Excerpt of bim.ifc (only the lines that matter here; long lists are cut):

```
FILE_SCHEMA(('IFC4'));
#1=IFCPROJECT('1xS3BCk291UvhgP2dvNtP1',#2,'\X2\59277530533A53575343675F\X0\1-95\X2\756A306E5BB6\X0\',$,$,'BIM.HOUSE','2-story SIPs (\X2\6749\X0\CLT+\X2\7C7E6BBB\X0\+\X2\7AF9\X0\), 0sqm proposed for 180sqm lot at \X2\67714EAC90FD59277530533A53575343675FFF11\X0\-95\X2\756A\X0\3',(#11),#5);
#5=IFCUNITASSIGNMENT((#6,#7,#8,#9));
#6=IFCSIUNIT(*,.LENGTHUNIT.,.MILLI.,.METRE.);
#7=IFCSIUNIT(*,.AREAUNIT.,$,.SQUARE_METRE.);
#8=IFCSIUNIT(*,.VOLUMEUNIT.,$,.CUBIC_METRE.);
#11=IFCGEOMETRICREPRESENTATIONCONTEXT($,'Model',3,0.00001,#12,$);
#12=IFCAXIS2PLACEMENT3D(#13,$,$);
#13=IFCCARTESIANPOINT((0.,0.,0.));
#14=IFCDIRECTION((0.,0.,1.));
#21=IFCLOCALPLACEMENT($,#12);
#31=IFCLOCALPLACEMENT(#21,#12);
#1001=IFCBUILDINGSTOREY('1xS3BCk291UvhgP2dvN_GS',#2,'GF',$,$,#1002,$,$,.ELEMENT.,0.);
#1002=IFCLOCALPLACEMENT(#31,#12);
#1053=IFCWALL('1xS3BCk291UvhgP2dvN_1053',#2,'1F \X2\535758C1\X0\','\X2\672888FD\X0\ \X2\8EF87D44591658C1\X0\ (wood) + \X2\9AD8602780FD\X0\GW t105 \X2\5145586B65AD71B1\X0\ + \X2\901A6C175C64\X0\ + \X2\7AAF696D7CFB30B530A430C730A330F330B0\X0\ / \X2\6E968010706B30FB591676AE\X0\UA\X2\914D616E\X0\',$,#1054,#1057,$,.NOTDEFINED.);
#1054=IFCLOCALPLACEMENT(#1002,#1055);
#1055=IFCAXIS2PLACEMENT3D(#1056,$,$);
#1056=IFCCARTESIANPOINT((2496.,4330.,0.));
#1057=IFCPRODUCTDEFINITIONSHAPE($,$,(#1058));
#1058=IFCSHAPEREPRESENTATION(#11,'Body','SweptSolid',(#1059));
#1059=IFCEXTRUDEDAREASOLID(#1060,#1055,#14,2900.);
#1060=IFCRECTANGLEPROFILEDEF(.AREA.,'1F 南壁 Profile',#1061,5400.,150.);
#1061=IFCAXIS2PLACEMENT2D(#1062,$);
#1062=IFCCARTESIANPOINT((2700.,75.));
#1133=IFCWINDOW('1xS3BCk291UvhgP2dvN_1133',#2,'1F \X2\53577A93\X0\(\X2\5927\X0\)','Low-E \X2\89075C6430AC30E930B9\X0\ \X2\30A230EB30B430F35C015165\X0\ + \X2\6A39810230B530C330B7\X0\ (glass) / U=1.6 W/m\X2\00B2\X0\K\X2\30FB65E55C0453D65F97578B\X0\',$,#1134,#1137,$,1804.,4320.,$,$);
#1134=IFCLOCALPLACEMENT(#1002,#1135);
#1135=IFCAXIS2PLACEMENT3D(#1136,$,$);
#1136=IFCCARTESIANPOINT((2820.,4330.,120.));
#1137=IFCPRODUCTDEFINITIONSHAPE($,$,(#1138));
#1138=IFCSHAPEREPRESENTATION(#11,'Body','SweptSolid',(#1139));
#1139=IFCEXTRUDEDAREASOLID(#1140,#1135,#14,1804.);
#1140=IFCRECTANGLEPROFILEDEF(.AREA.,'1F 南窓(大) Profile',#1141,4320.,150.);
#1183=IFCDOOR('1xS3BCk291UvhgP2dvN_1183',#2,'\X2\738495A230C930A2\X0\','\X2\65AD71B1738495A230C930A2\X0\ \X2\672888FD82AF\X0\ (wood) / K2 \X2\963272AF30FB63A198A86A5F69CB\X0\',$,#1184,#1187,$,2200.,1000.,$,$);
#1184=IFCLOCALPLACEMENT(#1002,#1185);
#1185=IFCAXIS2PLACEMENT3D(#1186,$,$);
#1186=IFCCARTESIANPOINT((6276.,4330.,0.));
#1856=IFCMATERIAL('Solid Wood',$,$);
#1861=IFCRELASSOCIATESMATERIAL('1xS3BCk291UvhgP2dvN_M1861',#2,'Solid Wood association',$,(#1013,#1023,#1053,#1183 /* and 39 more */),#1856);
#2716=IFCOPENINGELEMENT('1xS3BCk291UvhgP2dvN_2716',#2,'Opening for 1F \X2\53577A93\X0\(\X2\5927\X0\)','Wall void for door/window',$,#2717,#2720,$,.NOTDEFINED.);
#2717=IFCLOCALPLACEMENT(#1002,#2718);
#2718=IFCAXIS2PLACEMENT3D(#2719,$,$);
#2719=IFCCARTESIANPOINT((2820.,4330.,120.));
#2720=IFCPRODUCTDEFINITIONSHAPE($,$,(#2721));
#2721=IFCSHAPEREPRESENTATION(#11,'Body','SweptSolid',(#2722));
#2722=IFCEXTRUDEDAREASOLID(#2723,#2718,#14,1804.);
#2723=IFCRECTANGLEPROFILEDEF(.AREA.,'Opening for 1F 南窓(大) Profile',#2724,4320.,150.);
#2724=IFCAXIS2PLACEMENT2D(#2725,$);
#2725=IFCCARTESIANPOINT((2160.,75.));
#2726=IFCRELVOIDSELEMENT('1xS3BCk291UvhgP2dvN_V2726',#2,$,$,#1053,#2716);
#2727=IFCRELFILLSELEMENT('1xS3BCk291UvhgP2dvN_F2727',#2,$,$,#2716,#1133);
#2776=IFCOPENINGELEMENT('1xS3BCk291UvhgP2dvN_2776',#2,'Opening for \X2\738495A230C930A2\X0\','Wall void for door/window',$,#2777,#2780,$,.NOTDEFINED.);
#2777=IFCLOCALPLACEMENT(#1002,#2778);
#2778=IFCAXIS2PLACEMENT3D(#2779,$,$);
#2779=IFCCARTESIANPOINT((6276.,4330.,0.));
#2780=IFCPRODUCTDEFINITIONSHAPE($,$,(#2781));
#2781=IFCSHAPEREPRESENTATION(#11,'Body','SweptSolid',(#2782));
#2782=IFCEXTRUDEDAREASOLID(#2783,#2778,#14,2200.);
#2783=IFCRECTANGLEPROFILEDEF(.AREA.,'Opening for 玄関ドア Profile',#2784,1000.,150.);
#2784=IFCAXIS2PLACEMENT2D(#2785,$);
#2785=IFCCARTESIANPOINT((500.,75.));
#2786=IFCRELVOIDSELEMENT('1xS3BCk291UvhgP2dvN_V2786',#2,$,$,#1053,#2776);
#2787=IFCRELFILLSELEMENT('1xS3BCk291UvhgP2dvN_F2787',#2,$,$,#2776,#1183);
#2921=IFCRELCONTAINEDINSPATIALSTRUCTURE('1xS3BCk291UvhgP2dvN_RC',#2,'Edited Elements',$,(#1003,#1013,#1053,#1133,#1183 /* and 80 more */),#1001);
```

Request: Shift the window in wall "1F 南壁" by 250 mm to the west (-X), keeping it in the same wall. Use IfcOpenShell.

```python
import ifcopenshell
import ifcopenshell.api.geometry
import ifcopenshell.util.placement

model = ifcopenshell.open("bim.ifc")

window = model.by_id(1133)
opening = window.FillsVoids[0].RelatingOpeningElement
wall = opening.VoidsElements[0].RelatingBuildingElement

wall_matrix = ifcopenshell.util.placement.get_local_placement(wall.ObjectPlacement)
shift = wall_matrix[:3, 0] * -250.0
before = ifcopenshell.util.placement.get_local_placement(window.ObjectPlacement)[:3, 3].copy()

# The window is not placed relative to its opening, so move both.
for product in (opening, window):
    matrix = ifcopenshell.util.placement.get_local_placement(product.ObjectPlacement)
    matrix[:3, 3] += shift
    ifcopenshell.api.geometry.edit_object_placement(model, product=product, matrix=matrix, is_si=False)

after = ifcopenshell.util.placement.get_local_placement(window.ObjectPlacement)[:3, 3]
print("window moved by", (after - before).round(3) + 0.0)

model.write("bim-out.ifc")
```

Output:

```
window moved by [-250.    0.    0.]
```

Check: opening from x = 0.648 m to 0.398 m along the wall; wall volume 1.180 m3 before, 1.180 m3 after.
